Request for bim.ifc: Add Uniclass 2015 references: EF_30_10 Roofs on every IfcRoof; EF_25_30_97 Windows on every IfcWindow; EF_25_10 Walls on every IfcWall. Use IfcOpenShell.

First a look at what the model holds.

```python
import ifcopenshell

model = ifcopenshell.open("bim.ifc")
print(model.schema)
print("classifications:", [c.Name for c in model.by_type("IfcClassification")])
for ifc_class in ("IfcDoor", "IfcRoof", "IfcStair", "IfcWall", "IfcWindow"):
    print(ifc_class, len(model.by_type(ifc_class)))
```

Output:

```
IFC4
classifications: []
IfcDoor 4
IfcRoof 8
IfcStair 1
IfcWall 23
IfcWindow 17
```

```python
import ifcopenshell
import ifcopenshell.api.classification

model = ifcopenshell.open("bim.ifc")

system = ifcopenshell.api.classification.add_classification(model, classification="Uniclass 2015")

codes = {
    "IfcRoof": ("EF_30_10", "Roofs"),
    "IfcWindow": ("EF_25_30_97", "Windows"),
    "IfcWall": ("EF_25_10", "Walls"),
}
for ifc_class, (code, name) in codes.items():
    products = model.by_type(ifc_class)
    ifcopenshell.api.classification.add_reference(
        model, products=products, classification=system, identification=code, name=name
    )
    print(code, len(products))

model.write("bim_v2.ifc")
```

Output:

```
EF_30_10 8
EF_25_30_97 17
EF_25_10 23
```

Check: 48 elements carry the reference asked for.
